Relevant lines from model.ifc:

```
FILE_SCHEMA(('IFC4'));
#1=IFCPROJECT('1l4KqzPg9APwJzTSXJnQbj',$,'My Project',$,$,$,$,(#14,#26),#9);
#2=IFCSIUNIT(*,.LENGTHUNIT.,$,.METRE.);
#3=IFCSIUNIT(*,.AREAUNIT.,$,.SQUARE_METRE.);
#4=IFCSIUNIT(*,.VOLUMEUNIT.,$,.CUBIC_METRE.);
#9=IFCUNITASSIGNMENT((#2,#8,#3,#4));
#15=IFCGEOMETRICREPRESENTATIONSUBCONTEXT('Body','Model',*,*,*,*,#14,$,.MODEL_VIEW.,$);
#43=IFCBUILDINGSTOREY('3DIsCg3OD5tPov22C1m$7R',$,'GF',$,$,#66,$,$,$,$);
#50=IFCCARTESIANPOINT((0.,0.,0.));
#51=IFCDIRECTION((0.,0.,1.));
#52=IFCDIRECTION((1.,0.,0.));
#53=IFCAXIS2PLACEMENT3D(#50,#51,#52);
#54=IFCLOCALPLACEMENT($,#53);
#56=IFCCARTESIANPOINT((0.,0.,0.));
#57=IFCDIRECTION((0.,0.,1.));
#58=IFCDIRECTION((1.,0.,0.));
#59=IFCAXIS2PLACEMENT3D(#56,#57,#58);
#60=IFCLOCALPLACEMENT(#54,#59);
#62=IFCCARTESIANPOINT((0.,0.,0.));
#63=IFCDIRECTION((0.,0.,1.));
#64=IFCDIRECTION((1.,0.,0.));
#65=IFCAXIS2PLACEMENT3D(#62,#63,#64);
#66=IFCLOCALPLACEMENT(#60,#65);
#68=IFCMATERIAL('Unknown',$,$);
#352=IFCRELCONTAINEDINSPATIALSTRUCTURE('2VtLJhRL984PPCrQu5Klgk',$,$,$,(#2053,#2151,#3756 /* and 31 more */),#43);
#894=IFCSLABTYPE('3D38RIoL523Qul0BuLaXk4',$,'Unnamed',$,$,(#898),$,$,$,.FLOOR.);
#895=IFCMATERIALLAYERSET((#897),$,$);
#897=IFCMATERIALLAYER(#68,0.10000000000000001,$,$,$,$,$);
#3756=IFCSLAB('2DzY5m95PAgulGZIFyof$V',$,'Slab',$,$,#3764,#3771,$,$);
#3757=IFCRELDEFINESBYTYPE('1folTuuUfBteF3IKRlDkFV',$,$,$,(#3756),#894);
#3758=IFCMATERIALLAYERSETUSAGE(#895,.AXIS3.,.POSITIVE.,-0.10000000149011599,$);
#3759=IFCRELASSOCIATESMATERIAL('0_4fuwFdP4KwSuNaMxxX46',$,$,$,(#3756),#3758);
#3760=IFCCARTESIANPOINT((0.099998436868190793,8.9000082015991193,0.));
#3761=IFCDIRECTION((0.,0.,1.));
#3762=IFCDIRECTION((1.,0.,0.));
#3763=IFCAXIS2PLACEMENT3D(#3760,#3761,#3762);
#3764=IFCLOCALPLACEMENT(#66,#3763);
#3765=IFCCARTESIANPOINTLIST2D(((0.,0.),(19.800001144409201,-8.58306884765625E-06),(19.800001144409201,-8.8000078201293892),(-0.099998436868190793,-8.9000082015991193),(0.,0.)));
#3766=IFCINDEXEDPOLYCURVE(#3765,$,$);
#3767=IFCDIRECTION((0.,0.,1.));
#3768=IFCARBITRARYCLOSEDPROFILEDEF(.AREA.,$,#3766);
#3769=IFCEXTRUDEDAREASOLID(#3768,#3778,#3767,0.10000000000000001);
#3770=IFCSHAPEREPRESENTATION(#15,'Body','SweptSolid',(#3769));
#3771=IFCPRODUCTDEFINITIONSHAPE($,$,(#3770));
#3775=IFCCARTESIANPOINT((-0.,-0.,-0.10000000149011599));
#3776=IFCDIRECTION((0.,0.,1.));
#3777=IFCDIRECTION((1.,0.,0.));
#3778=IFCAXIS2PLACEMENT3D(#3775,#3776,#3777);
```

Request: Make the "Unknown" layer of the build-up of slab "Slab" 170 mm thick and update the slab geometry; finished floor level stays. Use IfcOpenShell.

```python
import ifcopenshell
import ifcopenshell.util.element
import ifcopenshell.util.representation

model = ifcopenshell.open("model.ifc")

layer_set = model.by_id(895)
layer = next(l for l in layer_set.MaterialLayers if l.Material and l.Material.Name == "Unknown")
change = 0.17 - layer.LayerThickness
layer.LayerThickness += change

# Geometry does not follow the layer set by itself.
slabs = [e for e in ifcopenshell.util.element.get_elements_by_material(model, layer_set) if e.is_a("IfcSlab")]
for slab in sorted(slabs, key=lambda e: e.id()):
    body = ifcopenshell.util.representation.get_representation(slab, "Model", "Body")
    solid = body.Items[0]
    old_depth = solid.Depth
    solid.Depth += change
    # Extruded upwards: lower the start of the extrusion so the top stays.
    x, y, z = solid.Position.Location.Coordinates
    solid.Position.Location = model.createIfcCartesianPoint((x, y, z - change))
    print(slab.id(), f"{old_depth:g} -> {solid.Depth:g}")

# The layers are counted up from the underside, which has moved.
for usage in {ifcopenshell.util.element.get_material(slab) for slab in slabs}:
    usage.OffsetFromReferenceLine -= change

model.write("model_v2.ifc")
```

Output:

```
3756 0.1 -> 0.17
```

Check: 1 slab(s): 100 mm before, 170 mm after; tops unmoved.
